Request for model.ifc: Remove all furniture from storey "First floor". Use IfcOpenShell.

First a look at what the model holds.

```python
import ifcopenshell
import ifcopenshell.util.element

model = ifcopenshell.open("model.ifc")
print(model.schema)
storey = next(s for s in model.by_type("IfcBuildingStorey") if s.Name == "First floor")
furniture = [e for e in ifcopenshell.util.element.get_decomposition(storey) if e.is_a("IfcFurnishingElement")]
seen = {}
for e in furniture:
    element_type = ifcopenshell.util.element.get_type(e)
    name = element_type.Name if element_type not in (None, e) else None
    seen[name] = seen.get(name, 0) + 1
for name, count in sorted(seen.items(), key=str):
    print(count, "x", name)
```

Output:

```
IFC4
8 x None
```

```python
import ifcopenshell
import ifcopenshell.api.root
import ifcopenshell.util.element

model = ifcopenshell.open("model.ifc")

storey = next(s for s in model.by_type("IfcBuildingStorey") if s.Name == "First floor")
furniture = [e for e in ifcopenshell.util.element.get_decomposition(storey) if e.is_a("IfcFurnishingElement")]

for e in furniture:
    ifcopenshell.api.root.remove_product(model, product=e)
print(len(furniture), "removed")

model.write("model_updated.ifc")
```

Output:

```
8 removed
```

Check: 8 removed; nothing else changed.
